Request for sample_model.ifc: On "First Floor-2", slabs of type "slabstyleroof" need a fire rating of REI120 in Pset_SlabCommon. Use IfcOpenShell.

First a look at what the model holds.

```python
import ifcopenshell
import ifcopenshell.util.element

model = ifcopenshell.open("sample_model.ifc")
print(model.schema)
storey = next(s for s in model.by_type("IfcBuildingStorey") if s.Name == "First Floor-2")
slabs = [e for e in ifcopenshell.util.element.get_decomposition(storey) if e.is_a("IfcSlab")]
seen = {}
for e in slabs:
    element_type = ifcopenshell.util.element.get_type(e)
    key = (element_type.Name if element_type != e and element_type else None, ifcopenshell.util.element.get_pset(e, "Pset_SlabCommon", "FireRating"))
    seen[key] = seen.get(key, 0) + 1
for (name, value), count in sorted(seen.items(), key=str):
    print(count, "x", name, "|", value)
```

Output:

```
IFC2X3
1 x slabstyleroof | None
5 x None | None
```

```python
import ifcopenshell
import ifcopenshell.api.pset
import ifcopenshell.util.element

model = ifcopenshell.open("sample_model.ifc")

storey = next(s for s in model.by_type("IfcBuildingStorey") if s.Name == "First Floor-2")
slabs = [e for e in ifcopenshell.util.element.get_decomposition(storey) if e.is_a("IfcSlab")]

count = 0
for e in slabs:
    element_type = ifcopenshell.util.element.get_type(e)
    if element_type in (None, e) or element_type.Name != "slabstyleroof":
        continue
    # add_pset returns the element's existing set when there is one.
    pset = ifcopenshell.api.pset.add_pset(model, product=e, name="Pset_SlabCommon")
    ifcopenshell.api.pset.edit_pset(model, pset=pset, properties={"FireRating": "REI120"})
    count += 1

print(count, "slabs updated")

model.write("sample_model_v2.ifc")
```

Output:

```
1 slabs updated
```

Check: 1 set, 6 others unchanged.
